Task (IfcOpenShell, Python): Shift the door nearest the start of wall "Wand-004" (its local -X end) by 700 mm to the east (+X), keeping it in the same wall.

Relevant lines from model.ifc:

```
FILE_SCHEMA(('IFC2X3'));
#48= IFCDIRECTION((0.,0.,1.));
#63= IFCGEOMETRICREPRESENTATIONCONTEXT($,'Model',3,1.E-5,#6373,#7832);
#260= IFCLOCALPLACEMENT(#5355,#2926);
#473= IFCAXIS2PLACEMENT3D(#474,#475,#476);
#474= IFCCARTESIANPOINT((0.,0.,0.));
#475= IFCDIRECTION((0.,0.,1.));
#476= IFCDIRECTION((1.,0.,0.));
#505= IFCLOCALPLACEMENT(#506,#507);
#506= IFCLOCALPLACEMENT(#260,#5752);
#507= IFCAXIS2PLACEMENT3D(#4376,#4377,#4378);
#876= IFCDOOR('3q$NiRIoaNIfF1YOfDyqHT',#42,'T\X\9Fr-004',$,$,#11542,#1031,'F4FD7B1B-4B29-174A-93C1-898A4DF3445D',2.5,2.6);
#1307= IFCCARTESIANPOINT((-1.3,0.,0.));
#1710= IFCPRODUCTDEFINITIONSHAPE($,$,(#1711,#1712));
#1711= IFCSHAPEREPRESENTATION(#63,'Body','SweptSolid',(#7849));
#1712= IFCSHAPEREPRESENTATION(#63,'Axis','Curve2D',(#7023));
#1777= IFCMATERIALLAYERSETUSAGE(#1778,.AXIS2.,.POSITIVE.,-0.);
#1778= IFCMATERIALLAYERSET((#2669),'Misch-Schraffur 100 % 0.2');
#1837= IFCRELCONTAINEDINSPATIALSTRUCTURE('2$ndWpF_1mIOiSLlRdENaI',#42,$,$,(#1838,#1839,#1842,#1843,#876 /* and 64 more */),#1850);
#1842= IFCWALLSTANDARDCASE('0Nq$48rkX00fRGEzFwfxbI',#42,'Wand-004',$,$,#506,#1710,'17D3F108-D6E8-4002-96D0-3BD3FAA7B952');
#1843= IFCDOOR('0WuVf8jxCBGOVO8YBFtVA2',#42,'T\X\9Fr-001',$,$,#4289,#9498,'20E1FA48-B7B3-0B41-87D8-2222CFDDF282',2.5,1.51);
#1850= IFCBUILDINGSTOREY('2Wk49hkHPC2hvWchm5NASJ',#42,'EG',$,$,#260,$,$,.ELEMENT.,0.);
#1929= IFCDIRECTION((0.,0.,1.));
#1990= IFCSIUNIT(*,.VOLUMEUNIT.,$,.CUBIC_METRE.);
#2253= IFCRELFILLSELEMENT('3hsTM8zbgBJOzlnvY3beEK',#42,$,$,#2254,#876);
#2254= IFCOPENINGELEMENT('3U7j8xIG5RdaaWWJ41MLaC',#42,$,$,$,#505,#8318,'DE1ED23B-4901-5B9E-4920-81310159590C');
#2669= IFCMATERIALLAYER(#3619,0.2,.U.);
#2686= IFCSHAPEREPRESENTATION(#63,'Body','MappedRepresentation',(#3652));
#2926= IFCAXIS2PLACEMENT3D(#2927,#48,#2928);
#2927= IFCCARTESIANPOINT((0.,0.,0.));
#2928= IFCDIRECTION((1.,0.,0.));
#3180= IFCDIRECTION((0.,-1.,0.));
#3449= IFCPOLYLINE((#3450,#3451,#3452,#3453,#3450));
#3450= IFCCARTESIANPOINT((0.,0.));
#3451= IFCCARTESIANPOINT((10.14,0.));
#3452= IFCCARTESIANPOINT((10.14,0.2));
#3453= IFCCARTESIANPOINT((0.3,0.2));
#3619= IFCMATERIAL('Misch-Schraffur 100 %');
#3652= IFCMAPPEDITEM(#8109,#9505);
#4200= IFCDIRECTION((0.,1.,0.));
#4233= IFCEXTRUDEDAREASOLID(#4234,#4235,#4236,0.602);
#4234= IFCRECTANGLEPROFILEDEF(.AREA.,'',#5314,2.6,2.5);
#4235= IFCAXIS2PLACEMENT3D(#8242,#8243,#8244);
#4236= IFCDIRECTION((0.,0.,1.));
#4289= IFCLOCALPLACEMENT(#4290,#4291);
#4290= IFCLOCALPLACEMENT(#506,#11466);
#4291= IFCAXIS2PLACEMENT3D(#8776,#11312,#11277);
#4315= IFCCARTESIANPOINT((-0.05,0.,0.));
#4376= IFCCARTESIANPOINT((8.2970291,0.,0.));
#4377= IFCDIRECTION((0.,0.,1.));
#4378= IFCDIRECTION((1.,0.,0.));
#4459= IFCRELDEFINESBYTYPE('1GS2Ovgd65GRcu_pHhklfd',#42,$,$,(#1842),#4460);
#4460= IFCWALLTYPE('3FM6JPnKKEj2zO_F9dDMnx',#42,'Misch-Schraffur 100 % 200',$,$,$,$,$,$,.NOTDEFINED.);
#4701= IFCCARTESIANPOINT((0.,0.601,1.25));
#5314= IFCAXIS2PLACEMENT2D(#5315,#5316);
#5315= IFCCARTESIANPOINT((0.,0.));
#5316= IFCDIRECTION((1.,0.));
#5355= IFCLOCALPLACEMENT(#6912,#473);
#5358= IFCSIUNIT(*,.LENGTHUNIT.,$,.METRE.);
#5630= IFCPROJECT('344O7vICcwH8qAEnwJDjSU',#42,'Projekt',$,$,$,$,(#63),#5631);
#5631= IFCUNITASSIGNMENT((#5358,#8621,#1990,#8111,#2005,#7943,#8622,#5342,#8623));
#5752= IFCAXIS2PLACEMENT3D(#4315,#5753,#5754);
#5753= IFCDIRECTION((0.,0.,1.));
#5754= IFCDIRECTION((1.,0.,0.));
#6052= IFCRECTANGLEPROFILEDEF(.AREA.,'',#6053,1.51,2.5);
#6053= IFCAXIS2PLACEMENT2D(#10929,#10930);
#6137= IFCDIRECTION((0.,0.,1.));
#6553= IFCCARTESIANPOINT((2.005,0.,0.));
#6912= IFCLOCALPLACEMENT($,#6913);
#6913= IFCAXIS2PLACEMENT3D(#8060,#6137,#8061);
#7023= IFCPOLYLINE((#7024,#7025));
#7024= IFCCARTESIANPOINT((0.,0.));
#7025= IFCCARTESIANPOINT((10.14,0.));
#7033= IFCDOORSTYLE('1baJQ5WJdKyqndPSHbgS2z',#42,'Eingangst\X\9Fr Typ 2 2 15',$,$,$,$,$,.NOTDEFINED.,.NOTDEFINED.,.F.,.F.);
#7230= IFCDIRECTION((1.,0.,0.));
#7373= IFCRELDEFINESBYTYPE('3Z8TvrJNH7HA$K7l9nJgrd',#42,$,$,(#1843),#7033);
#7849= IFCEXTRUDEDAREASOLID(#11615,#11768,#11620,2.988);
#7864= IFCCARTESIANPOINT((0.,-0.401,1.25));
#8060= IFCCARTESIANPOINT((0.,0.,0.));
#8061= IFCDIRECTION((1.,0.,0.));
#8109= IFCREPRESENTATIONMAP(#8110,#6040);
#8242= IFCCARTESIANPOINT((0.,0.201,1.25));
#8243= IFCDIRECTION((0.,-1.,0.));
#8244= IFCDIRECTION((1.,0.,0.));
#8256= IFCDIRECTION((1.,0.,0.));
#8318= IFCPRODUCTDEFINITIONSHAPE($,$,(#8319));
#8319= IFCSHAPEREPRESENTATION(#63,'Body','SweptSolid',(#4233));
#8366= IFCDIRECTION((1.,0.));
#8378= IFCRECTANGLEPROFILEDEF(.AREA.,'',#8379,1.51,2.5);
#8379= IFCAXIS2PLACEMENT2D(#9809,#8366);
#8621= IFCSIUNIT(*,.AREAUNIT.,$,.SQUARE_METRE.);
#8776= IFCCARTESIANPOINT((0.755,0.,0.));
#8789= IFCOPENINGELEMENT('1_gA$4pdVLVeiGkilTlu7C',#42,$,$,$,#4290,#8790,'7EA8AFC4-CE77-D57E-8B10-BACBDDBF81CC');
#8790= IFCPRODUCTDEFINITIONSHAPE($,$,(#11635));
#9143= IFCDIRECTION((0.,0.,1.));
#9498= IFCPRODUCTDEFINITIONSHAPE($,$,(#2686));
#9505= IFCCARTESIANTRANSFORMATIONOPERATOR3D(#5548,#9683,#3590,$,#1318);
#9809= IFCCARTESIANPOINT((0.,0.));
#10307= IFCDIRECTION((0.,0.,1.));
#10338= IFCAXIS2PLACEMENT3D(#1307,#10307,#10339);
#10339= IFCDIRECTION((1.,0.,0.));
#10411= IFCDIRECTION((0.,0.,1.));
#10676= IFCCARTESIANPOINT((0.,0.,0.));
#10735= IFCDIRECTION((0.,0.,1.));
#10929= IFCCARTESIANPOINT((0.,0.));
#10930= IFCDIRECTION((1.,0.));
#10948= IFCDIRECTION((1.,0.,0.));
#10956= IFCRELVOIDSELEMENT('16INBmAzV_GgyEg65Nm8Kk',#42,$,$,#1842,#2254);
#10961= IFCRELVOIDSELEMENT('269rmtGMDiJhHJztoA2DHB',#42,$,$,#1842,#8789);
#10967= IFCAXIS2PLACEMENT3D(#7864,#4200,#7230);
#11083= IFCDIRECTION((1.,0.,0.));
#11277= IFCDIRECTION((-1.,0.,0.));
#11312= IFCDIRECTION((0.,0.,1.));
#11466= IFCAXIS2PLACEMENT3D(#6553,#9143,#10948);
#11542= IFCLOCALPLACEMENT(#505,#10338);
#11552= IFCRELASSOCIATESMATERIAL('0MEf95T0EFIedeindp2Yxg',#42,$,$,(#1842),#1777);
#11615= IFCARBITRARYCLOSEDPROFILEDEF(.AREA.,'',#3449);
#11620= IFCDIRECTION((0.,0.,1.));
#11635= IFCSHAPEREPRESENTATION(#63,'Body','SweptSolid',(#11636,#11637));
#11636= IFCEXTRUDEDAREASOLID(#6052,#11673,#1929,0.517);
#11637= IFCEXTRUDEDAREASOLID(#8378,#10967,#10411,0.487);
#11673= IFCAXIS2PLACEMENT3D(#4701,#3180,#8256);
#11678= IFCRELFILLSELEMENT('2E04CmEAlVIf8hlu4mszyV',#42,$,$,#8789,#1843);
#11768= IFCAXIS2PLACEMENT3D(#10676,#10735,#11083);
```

```python
import ifcopenshell
import ifcopenshell.api.geometry
import ifcopenshell.util.placement
import ifcopenshell.util.unit

model = ifcopenshell.open("model.ifc")
unit_scale = ifcopenshell.util.unit.calculate_unit_scale(model)

door = model.by_guid("0WuVf8jxCBGOVO8YBFtVA2")
opening = door.FillsVoids[0].RelatingOpeningElement
wall = opening.VoidsElements[0].RelatingBuildingElement

wall_matrix = ifcopenshell.util.placement.get_local_placement(wall.ObjectPlacement)
shift = wall_matrix[:3, 0] * 0.7 / unit_scale
before = ifcopenshell.util.placement.get_local_placement(door.ObjectPlacement)[:3, 3].copy()

# The door is placed relative to its opening, so it follows when the opening moves.
matrix = ifcopenshell.util.placement.get_local_placement(opening.ObjectPlacement)
matrix[:3, 3] += shift
ifcopenshell.api.geometry.edit_object_placement(
    model, product=opening, matrix=matrix, is_si=False, should_transform_children=True
)

after = ifcopenshell.util.placement.get_local_placement(door.ObjectPlacement)[:3, 3]
print("door moved by", (after - before).round(3) + 0.0)

model.write("model_edited.ifc")
```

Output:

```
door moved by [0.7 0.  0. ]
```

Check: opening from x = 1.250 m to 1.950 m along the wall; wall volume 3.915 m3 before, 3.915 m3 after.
